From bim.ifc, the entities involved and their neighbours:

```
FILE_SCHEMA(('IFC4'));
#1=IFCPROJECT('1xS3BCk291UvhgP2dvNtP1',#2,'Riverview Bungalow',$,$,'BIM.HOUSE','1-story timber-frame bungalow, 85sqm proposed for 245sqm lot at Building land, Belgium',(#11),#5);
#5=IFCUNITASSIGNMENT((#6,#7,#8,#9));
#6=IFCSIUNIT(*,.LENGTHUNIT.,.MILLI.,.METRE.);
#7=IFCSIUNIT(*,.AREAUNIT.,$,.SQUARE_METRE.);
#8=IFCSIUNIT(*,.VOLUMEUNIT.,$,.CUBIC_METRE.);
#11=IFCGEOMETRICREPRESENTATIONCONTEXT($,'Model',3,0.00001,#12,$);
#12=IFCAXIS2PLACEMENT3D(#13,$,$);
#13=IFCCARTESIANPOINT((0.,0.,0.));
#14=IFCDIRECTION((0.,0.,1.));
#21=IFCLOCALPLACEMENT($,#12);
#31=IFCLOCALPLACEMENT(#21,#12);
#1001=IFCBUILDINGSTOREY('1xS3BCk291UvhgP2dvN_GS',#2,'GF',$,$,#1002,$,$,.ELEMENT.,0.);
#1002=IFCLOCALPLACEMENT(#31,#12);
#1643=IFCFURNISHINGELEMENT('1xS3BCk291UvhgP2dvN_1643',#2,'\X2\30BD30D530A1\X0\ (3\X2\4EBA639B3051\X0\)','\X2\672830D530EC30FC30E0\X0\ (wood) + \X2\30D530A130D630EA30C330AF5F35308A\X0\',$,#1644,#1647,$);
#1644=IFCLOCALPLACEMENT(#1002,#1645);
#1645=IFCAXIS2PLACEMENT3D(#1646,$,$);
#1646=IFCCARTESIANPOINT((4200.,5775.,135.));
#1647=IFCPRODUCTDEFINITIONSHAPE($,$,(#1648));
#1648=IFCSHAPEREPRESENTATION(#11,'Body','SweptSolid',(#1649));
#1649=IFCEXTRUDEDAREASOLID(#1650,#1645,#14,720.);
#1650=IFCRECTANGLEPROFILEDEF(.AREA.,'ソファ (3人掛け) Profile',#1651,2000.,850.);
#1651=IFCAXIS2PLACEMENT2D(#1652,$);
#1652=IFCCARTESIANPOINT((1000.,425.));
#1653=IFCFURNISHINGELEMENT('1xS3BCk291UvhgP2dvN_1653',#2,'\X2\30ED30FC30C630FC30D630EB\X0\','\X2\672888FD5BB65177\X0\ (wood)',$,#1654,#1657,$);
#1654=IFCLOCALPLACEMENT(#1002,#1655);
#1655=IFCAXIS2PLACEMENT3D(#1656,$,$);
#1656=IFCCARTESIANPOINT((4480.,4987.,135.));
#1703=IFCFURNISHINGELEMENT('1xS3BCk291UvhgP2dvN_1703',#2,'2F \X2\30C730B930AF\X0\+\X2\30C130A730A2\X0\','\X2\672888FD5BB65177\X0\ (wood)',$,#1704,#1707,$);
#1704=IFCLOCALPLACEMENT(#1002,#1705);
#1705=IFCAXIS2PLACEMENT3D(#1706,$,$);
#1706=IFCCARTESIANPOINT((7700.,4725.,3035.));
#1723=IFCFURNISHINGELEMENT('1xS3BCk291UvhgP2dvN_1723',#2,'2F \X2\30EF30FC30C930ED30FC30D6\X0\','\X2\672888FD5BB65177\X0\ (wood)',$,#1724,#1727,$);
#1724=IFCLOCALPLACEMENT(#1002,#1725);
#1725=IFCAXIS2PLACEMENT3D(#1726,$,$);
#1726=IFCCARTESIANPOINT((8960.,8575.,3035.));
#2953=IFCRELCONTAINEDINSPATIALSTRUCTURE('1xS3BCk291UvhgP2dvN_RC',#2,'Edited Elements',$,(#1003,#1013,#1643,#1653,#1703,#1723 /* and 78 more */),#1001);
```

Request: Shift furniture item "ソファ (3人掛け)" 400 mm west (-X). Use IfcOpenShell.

```python
import ifcopenshell
import ifcopenshell.api.geometry
import ifcopenshell.util.placement
import ifcopenshell.util.unit

model = ifcopenshell.open("bim.ifc")
unit_scale = ifcopenshell.util.unit.calculate_unit_scale(model)

item = model.by_id(1643)
matrix = ifcopenshell.util.placement.get_local_placement(item.ObjectPlacement)
matrix[0, 3] -= 0.4 / unit_scale
ifcopenshell.api.geometry.edit_object_placement(model, product=item, matrix=matrix, is_si=False)

print(ifcopenshell.util.placement.get_local_placement(item.ObjectPlacement).round(3) + 0.0)

model.write("bim_updated.ifc")
```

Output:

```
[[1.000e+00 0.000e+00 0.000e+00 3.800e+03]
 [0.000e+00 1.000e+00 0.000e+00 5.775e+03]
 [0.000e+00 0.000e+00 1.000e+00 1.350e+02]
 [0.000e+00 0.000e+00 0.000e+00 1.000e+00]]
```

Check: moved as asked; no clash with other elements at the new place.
